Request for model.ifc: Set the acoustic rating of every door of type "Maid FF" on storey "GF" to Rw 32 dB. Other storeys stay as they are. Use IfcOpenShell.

First a look at what the model holds.

```python
import ifcopenshell
import ifcopenshell.util.element

model = ifcopenshell.open("model.ifc")
print(model.schema)
storey = next(s for s in model.by_type("IfcBuildingStorey") if s.Name == "GF")
doors = [e for e in ifcopenshell.util.element.get_decomposition(storey) if e.is_a("IfcDoor")]
seen = {}
for e in doors:
    element_type = ifcopenshell.util.element.get_type(e)
    key = (element_type.Name if element_type != e and element_type else None, ifcopenshell.util.element.get_pset(e, "Pset_DoorCommon", "AcousticRating"))
    seen[key] = seen.get(key, 0) + 1
for (name, value), count in sorted(seen.items(), key=str):
    print(count, "x", name, "|", value)
```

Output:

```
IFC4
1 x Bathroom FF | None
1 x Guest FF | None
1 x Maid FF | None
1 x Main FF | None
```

```python
import ifcopenshell
import ifcopenshell.api.pset
import ifcopenshell.util.element

model = ifcopenshell.open("model.ifc")

storey = next(s for s in model.by_type("IfcBuildingStorey") if s.Name == "GF")
doors = [e for e in ifcopenshell.util.element.get_decomposition(storey) if e.is_a("IfcDoor")]

count = 0
for e in doors:
    element_type = ifcopenshell.util.element.get_type(e)
    if element_type in (None, e) or element_type.Name != "Maid FF":
        continue
    # add_pset returns the element's existing set when there is one.
    pset = ifcopenshell.api.pset.add_pset(model, product=e, name="Pset_DoorCommon")
    ifcopenshell.api.pset.edit_pset(model, pset=pset, properties={"AcousticRating": "Rw 32 dB"})
    count += 1

print(count, "doors updated")

model.write("model_edited.ifc")
```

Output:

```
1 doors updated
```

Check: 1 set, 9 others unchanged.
